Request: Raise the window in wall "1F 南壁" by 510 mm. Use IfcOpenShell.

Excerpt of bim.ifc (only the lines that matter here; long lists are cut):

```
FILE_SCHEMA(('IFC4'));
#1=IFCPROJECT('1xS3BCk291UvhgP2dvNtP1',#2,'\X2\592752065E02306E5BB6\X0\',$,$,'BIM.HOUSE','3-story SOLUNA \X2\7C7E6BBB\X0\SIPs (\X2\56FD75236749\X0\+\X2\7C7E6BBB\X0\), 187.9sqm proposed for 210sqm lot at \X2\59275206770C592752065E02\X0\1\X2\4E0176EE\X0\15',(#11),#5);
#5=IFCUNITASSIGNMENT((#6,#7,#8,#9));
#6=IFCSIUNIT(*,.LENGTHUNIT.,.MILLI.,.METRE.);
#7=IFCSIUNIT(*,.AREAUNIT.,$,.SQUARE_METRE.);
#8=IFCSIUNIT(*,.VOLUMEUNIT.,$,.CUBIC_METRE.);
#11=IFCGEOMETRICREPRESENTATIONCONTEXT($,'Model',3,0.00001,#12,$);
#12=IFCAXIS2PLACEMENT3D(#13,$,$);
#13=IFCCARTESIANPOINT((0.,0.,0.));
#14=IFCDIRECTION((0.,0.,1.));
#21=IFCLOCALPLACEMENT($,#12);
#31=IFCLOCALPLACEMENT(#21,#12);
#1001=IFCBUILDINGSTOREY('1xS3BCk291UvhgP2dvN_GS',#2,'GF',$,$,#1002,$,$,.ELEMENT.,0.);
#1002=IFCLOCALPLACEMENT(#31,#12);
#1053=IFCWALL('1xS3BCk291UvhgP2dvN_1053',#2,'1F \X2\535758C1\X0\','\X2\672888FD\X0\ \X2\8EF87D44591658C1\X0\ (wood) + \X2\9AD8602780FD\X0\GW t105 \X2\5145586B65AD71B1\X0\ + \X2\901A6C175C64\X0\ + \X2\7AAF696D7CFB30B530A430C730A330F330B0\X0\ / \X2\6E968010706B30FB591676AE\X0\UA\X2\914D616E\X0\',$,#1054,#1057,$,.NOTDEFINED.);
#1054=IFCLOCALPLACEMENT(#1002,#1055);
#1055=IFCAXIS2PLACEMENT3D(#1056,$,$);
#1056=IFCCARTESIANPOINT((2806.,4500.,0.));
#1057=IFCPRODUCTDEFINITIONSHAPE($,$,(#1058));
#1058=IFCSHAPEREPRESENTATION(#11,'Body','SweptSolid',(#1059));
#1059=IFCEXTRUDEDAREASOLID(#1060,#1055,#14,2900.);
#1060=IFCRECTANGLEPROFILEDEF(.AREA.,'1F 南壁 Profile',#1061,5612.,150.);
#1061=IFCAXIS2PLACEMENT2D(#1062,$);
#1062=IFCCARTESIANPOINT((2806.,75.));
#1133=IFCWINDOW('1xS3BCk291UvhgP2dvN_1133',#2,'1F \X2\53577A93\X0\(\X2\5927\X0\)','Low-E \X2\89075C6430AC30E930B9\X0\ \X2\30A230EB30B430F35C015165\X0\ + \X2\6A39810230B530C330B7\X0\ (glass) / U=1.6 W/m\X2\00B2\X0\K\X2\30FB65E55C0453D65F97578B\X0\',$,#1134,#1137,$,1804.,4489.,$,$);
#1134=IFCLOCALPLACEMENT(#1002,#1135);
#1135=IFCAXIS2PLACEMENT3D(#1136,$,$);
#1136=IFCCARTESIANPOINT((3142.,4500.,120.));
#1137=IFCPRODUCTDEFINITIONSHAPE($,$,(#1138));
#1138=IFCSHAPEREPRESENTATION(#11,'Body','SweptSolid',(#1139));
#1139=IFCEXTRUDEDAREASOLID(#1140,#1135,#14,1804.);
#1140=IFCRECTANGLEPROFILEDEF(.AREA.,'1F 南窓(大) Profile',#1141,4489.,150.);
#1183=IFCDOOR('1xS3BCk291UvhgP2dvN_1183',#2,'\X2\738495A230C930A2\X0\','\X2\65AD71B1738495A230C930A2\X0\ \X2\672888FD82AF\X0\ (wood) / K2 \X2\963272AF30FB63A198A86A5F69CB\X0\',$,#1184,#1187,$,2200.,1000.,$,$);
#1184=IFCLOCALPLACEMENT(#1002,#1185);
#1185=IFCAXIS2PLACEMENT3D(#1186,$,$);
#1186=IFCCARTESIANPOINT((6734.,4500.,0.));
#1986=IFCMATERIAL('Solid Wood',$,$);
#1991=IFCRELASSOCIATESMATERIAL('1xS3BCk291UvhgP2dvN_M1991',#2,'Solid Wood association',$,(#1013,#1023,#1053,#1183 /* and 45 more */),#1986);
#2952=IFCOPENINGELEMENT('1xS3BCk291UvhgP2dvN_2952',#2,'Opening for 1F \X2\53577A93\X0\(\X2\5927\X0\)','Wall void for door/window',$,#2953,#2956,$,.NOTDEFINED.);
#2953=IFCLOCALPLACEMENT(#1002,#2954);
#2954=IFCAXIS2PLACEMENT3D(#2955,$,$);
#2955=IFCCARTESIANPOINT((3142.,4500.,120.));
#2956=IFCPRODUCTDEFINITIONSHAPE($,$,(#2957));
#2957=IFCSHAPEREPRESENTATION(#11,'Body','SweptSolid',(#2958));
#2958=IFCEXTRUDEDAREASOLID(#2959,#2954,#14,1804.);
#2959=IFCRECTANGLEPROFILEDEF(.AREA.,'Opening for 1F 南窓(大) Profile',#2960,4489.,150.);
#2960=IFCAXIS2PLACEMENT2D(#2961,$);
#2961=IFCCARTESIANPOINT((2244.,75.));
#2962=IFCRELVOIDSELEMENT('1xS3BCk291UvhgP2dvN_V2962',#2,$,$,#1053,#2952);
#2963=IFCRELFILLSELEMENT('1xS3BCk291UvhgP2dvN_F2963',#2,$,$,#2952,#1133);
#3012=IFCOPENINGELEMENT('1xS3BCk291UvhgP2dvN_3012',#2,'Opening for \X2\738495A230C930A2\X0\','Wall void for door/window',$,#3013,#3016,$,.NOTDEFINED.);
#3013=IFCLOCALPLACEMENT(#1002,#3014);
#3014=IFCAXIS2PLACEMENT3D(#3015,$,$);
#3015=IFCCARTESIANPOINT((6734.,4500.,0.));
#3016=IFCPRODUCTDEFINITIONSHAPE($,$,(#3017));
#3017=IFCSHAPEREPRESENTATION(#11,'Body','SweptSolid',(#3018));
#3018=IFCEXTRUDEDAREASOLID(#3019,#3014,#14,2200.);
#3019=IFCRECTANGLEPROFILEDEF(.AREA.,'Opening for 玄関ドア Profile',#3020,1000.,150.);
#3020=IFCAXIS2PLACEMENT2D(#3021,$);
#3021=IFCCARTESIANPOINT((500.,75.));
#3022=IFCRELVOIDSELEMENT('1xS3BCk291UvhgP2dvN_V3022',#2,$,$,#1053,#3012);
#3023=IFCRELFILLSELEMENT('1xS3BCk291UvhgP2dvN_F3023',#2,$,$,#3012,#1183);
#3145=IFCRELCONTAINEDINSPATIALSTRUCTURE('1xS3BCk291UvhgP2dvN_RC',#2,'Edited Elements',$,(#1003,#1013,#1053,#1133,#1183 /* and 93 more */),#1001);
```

```python
import numpy as np
import ifcopenshell
import ifcopenshell.api.geometry
import ifcopenshell.util.placement
import ifcopenshell.util.unit

model = ifcopenshell.open("bim.ifc")
unit_scale = ifcopenshell.util.unit.calculate_unit_scale(model)

window = model.by_guid("1xS3BCk291UvhgP2dvN_1133")
opening = window.FillsVoids[0].RelatingOpeningElement
dz = 0.51 / unit_scale

shift = np.array([0.0, 0.0, dz])
# The window is not placed relative to its opening, so move both.
for product in (opening, window):
    matrix = ifcopenshell.util.placement.get_local_placement(product.ObjectPlacement)
    matrix[:3, 3] += shift
    ifcopenshell.api.geometry.edit_object_placement(model, product=product, matrix=matrix, is_si=False)

print(f"moved by {dz * unit_scale:+.3f} m")

model.write("bim_updated.ifc")
```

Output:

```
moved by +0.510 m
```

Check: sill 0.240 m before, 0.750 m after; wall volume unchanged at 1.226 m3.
